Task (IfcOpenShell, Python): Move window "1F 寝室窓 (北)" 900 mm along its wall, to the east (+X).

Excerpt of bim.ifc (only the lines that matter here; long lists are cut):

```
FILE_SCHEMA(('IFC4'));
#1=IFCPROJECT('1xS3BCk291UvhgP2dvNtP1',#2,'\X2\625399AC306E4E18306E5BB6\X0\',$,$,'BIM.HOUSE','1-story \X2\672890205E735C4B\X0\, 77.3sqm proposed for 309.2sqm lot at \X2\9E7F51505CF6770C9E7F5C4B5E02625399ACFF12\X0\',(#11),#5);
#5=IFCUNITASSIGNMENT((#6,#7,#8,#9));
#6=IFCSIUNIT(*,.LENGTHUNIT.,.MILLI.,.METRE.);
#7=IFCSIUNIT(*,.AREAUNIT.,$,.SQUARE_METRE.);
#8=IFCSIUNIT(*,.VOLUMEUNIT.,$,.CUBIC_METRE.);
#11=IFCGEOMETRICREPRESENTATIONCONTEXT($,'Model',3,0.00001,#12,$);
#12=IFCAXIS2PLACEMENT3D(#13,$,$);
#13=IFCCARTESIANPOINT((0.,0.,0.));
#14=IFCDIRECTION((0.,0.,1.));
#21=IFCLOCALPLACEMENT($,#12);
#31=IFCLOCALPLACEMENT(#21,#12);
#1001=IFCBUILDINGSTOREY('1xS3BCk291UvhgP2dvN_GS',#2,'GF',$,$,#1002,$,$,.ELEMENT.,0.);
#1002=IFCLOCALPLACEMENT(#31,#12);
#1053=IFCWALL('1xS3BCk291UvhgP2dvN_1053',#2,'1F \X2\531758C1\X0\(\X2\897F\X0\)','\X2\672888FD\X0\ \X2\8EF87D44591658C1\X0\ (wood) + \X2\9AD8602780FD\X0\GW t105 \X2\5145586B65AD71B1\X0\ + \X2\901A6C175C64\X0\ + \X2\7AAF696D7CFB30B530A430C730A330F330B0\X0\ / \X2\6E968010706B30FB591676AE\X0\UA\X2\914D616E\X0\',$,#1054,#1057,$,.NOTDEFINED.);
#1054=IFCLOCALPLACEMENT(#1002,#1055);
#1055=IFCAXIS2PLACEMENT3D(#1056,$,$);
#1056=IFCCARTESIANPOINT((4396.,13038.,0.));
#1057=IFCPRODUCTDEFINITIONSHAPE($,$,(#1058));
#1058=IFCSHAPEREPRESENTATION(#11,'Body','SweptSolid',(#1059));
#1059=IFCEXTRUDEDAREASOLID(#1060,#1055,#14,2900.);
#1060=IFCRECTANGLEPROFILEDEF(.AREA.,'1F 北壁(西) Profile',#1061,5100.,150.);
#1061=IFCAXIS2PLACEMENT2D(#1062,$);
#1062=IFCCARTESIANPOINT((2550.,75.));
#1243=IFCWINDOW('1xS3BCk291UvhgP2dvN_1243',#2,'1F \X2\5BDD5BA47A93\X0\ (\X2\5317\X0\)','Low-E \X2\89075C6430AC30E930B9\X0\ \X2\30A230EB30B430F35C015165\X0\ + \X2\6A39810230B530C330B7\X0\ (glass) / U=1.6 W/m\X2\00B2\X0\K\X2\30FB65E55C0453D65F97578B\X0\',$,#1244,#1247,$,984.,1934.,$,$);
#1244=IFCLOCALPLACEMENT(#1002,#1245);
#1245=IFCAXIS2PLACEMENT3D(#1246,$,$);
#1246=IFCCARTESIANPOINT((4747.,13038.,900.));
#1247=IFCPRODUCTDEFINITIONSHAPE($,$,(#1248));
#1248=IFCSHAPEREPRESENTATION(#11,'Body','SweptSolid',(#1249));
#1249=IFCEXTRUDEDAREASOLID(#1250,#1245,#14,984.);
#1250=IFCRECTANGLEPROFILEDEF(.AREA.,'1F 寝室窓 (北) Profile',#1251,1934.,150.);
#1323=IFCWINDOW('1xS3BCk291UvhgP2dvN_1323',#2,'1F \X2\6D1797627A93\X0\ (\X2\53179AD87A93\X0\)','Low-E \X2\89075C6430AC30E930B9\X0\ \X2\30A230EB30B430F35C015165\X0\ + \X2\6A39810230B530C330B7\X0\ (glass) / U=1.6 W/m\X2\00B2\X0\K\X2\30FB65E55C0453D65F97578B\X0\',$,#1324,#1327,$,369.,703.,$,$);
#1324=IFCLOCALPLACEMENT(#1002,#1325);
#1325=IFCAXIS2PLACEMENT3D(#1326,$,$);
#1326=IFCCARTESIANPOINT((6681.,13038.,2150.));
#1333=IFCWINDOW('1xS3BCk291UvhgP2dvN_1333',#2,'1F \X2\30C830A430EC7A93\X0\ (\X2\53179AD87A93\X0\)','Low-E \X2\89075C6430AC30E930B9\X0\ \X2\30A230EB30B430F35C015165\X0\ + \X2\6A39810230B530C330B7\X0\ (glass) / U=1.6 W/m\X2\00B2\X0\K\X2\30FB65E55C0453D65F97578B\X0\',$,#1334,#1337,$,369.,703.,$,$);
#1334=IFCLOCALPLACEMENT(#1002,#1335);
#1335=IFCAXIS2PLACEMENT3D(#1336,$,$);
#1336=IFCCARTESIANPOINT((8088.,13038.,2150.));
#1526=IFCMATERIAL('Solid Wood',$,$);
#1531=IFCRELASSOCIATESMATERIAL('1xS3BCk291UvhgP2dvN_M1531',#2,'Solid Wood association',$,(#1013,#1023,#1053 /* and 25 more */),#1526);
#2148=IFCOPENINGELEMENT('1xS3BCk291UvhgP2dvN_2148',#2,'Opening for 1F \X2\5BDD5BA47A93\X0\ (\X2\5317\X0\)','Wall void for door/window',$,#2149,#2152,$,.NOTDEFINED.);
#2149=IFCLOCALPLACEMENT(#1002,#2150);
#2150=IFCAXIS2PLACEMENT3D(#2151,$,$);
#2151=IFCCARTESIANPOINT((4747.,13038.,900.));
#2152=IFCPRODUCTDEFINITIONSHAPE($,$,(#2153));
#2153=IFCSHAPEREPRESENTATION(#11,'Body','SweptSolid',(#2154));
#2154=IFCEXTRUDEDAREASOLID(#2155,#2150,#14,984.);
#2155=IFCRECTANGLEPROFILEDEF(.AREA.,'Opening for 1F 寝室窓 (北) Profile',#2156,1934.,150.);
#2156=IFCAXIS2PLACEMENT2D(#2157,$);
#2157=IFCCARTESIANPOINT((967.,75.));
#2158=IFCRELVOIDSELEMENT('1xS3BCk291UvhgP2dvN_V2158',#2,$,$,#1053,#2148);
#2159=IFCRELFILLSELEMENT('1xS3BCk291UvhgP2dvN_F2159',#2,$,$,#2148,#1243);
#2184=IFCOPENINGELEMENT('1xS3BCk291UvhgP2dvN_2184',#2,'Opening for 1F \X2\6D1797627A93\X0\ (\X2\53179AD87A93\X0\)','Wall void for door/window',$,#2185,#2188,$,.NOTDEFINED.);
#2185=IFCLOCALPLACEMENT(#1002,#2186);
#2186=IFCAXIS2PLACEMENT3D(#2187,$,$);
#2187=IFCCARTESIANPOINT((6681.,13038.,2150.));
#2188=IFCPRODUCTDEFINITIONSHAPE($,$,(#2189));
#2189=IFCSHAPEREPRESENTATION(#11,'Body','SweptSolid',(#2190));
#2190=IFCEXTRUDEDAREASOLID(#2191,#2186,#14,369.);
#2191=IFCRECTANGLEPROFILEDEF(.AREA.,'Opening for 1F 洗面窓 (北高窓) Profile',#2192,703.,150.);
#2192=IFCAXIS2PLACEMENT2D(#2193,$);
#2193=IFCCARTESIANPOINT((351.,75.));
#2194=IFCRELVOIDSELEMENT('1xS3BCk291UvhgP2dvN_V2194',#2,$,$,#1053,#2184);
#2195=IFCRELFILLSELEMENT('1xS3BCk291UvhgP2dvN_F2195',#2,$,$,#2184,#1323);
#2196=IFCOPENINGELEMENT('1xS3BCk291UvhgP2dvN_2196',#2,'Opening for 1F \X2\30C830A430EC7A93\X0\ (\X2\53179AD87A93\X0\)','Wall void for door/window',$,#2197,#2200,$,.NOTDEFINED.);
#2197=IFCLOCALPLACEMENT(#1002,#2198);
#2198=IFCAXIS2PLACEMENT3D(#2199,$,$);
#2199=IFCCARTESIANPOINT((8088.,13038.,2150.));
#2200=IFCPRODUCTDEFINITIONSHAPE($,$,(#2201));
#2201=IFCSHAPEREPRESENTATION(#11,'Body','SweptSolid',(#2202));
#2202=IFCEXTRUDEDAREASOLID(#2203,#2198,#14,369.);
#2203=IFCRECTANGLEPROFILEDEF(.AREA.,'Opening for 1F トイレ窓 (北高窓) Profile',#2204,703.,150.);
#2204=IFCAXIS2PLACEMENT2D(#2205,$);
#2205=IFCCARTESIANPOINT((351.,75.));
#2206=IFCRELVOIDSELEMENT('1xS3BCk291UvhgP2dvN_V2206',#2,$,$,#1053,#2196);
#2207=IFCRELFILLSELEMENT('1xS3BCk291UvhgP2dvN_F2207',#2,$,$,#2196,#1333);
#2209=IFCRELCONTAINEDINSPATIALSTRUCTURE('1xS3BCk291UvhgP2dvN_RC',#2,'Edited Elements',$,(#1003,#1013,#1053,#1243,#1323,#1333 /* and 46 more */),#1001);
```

```python
import ifcopenshell
import ifcopenshell.api.geometry
import ifcopenshell.util.placement

model = ifcopenshell.open("bim.ifc")

window = model.by_guid("1xS3BCk291UvhgP2dvN_1243")
opening = window.FillsVoids[0].RelatingOpeningElement
wall = opening.VoidsElements[0].RelatingBuildingElement

wall_matrix = ifcopenshell.util.placement.get_local_placement(wall.ObjectPlacement)
shift = wall_matrix[:3, 0] * 900.0
before = ifcopenshell.util.placement.get_local_placement(window.ObjectPlacement)[:3, 3].copy()

# The window is not placed relative to its opening, so move both.
for product in (opening, window):
    matrix = ifcopenshell.util.placement.get_local_placement(product.ObjectPlacement)
    matrix[:3, 3] += shift
    ifcopenshell.api.geometry.edit_object_placement(model, product=product, matrix=matrix, is_si=False)

after = ifcopenshell.util.placement.get_local_placement(window.ObjectPlacement)[:3, 3]
print("window moved by", (after - before).round(3) + 0.0)

model.write("bim_updated.ifc")
```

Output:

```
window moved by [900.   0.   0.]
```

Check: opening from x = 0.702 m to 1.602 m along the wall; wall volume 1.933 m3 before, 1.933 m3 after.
